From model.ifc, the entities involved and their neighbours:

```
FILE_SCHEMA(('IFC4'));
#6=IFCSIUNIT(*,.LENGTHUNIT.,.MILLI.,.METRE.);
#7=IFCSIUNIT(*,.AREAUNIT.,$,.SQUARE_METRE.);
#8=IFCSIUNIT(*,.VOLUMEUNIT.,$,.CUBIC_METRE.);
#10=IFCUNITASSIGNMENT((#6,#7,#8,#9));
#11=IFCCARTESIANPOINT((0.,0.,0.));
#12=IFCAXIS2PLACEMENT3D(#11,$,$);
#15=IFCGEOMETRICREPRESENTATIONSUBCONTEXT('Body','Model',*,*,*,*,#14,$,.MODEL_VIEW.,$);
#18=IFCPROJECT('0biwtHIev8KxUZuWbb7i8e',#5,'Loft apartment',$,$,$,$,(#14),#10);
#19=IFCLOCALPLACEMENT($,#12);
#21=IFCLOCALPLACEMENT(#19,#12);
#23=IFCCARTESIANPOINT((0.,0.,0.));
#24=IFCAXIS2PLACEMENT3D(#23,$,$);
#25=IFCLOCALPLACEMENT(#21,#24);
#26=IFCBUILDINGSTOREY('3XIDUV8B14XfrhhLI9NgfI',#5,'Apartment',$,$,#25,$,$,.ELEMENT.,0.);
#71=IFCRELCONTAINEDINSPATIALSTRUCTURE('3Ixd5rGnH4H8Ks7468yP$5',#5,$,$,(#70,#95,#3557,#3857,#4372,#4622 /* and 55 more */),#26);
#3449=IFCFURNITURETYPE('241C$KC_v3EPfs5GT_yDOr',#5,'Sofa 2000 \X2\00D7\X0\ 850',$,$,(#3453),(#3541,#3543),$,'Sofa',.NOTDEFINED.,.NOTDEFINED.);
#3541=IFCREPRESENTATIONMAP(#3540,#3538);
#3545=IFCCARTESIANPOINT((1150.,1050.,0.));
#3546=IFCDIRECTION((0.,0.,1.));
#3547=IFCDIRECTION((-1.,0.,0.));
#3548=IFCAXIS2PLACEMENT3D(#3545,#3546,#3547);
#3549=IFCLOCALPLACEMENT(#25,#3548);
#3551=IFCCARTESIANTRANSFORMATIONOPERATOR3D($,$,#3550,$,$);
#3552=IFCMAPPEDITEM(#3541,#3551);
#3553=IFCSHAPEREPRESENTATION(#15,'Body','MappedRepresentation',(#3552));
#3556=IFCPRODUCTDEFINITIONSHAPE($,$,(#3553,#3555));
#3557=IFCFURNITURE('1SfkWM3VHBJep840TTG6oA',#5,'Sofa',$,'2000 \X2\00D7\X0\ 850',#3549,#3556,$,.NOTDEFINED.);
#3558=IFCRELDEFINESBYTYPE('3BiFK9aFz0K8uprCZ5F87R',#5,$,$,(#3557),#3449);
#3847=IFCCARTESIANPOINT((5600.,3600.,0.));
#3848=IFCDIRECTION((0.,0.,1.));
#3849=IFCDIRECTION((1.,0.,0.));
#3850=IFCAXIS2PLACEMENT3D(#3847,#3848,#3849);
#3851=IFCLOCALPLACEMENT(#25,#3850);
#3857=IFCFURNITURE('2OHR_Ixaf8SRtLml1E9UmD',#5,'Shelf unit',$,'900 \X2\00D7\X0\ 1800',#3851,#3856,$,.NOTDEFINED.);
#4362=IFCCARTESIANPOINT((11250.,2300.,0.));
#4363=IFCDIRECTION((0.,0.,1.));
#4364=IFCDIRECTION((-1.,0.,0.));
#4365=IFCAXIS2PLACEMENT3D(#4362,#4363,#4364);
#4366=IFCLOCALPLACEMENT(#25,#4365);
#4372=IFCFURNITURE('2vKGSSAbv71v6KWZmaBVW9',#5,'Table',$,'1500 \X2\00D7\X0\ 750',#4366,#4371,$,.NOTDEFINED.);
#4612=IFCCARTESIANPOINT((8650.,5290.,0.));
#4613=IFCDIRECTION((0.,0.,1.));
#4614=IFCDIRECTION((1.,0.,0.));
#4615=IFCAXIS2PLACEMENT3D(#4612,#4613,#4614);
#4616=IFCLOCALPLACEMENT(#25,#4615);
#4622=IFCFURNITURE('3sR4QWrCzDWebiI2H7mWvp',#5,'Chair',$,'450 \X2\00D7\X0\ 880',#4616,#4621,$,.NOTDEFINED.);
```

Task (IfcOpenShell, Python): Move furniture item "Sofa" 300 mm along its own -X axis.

```python
import ifcopenshell
import ifcopenshell.api.geometry
import ifcopenshell.util.placement

model = ifcopenshell.open("model.ifc")

item = model.by_guid("1SfkWM3VHBJep840TTG6oA")
matrix = ifcopenshell.util.placement.get_local_placement(item.ObjectPlacement)
matrix[:3, 3] -= matrix[:3, 0] * 300.0
ifcopenshell.api.geometry.edit_object_placement(model, product=item, matrix=matrix, is_si=False)

print(ifcopenshell.util.placement.get_local_placement(item.ObjectPlacement).round(3) + 0.0)

model.write("model_v2.ifc")
```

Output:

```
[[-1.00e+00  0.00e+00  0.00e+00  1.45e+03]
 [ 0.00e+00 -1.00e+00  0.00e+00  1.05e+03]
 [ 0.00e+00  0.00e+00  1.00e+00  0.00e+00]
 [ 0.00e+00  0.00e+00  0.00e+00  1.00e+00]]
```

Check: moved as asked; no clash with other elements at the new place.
